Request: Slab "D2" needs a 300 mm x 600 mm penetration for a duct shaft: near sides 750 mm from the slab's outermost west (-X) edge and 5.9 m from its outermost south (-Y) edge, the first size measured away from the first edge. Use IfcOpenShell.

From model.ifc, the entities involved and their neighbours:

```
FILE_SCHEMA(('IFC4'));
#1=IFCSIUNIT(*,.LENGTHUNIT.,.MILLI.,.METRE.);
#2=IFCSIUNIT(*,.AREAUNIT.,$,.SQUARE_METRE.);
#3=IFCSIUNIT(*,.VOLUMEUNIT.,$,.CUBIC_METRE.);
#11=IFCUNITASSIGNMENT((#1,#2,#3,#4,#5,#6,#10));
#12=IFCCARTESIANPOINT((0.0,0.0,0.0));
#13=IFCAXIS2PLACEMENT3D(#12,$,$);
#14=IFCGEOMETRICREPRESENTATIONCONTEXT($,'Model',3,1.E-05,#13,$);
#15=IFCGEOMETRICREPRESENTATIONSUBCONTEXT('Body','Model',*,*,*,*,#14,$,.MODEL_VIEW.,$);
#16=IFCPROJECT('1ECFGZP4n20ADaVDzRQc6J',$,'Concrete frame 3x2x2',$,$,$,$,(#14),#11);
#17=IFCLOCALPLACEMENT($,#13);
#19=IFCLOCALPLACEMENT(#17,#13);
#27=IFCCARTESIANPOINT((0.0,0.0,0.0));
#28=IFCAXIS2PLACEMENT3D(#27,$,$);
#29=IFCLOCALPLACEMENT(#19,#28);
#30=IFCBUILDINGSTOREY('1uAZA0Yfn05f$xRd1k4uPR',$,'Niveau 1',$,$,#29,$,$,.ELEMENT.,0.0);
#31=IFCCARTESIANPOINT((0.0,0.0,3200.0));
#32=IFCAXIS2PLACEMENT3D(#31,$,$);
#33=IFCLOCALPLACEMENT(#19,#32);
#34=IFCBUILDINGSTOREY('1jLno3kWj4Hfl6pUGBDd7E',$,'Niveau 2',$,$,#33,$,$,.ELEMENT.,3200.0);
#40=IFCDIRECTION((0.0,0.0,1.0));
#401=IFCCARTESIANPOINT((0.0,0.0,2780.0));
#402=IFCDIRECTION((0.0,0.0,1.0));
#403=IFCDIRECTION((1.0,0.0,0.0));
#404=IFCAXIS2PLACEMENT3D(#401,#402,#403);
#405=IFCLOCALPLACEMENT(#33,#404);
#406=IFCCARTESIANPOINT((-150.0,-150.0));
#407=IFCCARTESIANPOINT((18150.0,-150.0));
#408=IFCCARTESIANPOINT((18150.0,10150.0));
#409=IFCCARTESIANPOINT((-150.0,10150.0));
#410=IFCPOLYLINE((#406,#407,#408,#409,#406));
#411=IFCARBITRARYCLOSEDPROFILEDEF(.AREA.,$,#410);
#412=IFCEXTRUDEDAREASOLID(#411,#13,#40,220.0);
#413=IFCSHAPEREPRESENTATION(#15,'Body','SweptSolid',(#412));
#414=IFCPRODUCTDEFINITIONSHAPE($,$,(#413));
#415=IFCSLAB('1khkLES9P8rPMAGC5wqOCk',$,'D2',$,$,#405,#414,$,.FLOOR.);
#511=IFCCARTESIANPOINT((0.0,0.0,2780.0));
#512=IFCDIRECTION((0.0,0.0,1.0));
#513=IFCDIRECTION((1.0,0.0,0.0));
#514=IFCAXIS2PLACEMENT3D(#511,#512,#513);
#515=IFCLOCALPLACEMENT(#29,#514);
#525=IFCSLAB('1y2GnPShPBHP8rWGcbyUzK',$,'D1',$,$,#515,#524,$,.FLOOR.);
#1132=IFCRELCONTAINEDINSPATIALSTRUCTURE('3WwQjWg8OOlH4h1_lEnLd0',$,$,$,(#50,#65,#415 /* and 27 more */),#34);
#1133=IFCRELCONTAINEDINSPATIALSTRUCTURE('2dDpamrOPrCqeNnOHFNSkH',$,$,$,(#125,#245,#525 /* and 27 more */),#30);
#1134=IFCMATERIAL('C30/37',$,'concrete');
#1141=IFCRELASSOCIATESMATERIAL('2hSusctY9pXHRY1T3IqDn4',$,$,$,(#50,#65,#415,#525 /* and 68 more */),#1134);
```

```python
import numpy as np
import ifcopenshell
import ifcopenshell.api.feature
import ifcopenshell.api.geometry
import ifcopenshell.api.root
import ifcopenshell.geom
import ifcopenshell.util.placement
import ifcopenshell.util.representation
import ifcopenshell.util.shape
import ifcopenshell.util.unit

model = ifcopenshell.open("model.ifc")
unit_scale = ifcopenshell.util.unit.calculate_unit_scale(model)
settings = ifcopenshell.geom.settings()


def volume(element):
    """Net volume in cubic metres, openings subtracted."""
    shape = ifcopenshell.geom.create_shape(settings, element)
    return ifcopenshell.util.shape.get_volume(shape.geometry)


slab = model.by_guid("1khkLES9P8rPMAGC5wqOCk")
before = volume(slab)

# Extent in the slab's own axes, in metres. The edges named are its -X and -Y sides.
slab_shape = ifcopenshell.geom.create_shape(settings, slab)
vertices = ifcopenshell.util.shape.get_vertices(slab_shape.geometry)
x_min, y_min, bottom = vertices.min(axis=0)
top = vertices[:, 2].max()

opening = ifcopenshell.api.root.create_entity(model, ifc_class="IfcOpeningElement", name="Duct shaft opening", predefined_type="OPENING")
context = ifcopenshell.util.representation.get_context(model, "Model", "Body", "MODEL_VIEW")
width, depth = 0.3, 0.6
outline = [(0.0, 0.0), (width, 0.0), (width, depth), (0.0, depth), (0.0, 0.0)]
# Overshoot both faces by 50 mm so the cut is clean.
shape = ifcopenshell.api.geometry.add_slab_representation(
    model, context=context, depth=top - bottom + 0.1, polyline=outline
)
ifcopenshell.api.geometry.assign_representation(model, product=opening, representation=shape)

matrix = ifcopenshell.util.placement.get_local_placement(slab.ObjectPlacement)
matrix[:, 3] = matrix @ np.append(np.array([x_min + 0.75, y_min + 5.9, bottom - 0.05]) / unit_scale, 1.0)
ifcopenshell.api.geometry.edit_object_placement(model, product=opening, matrix=matrix, is_si=False)
ifcopenshell.api.feature.add_feature(model, feature=opening, element=slab)

after = volume(slab)

print(f"slab volume {before:.3f} -> {after:.3f} m3")

model.write("model_updated.ifc")
```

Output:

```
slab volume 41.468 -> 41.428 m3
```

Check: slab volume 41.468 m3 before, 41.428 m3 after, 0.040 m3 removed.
